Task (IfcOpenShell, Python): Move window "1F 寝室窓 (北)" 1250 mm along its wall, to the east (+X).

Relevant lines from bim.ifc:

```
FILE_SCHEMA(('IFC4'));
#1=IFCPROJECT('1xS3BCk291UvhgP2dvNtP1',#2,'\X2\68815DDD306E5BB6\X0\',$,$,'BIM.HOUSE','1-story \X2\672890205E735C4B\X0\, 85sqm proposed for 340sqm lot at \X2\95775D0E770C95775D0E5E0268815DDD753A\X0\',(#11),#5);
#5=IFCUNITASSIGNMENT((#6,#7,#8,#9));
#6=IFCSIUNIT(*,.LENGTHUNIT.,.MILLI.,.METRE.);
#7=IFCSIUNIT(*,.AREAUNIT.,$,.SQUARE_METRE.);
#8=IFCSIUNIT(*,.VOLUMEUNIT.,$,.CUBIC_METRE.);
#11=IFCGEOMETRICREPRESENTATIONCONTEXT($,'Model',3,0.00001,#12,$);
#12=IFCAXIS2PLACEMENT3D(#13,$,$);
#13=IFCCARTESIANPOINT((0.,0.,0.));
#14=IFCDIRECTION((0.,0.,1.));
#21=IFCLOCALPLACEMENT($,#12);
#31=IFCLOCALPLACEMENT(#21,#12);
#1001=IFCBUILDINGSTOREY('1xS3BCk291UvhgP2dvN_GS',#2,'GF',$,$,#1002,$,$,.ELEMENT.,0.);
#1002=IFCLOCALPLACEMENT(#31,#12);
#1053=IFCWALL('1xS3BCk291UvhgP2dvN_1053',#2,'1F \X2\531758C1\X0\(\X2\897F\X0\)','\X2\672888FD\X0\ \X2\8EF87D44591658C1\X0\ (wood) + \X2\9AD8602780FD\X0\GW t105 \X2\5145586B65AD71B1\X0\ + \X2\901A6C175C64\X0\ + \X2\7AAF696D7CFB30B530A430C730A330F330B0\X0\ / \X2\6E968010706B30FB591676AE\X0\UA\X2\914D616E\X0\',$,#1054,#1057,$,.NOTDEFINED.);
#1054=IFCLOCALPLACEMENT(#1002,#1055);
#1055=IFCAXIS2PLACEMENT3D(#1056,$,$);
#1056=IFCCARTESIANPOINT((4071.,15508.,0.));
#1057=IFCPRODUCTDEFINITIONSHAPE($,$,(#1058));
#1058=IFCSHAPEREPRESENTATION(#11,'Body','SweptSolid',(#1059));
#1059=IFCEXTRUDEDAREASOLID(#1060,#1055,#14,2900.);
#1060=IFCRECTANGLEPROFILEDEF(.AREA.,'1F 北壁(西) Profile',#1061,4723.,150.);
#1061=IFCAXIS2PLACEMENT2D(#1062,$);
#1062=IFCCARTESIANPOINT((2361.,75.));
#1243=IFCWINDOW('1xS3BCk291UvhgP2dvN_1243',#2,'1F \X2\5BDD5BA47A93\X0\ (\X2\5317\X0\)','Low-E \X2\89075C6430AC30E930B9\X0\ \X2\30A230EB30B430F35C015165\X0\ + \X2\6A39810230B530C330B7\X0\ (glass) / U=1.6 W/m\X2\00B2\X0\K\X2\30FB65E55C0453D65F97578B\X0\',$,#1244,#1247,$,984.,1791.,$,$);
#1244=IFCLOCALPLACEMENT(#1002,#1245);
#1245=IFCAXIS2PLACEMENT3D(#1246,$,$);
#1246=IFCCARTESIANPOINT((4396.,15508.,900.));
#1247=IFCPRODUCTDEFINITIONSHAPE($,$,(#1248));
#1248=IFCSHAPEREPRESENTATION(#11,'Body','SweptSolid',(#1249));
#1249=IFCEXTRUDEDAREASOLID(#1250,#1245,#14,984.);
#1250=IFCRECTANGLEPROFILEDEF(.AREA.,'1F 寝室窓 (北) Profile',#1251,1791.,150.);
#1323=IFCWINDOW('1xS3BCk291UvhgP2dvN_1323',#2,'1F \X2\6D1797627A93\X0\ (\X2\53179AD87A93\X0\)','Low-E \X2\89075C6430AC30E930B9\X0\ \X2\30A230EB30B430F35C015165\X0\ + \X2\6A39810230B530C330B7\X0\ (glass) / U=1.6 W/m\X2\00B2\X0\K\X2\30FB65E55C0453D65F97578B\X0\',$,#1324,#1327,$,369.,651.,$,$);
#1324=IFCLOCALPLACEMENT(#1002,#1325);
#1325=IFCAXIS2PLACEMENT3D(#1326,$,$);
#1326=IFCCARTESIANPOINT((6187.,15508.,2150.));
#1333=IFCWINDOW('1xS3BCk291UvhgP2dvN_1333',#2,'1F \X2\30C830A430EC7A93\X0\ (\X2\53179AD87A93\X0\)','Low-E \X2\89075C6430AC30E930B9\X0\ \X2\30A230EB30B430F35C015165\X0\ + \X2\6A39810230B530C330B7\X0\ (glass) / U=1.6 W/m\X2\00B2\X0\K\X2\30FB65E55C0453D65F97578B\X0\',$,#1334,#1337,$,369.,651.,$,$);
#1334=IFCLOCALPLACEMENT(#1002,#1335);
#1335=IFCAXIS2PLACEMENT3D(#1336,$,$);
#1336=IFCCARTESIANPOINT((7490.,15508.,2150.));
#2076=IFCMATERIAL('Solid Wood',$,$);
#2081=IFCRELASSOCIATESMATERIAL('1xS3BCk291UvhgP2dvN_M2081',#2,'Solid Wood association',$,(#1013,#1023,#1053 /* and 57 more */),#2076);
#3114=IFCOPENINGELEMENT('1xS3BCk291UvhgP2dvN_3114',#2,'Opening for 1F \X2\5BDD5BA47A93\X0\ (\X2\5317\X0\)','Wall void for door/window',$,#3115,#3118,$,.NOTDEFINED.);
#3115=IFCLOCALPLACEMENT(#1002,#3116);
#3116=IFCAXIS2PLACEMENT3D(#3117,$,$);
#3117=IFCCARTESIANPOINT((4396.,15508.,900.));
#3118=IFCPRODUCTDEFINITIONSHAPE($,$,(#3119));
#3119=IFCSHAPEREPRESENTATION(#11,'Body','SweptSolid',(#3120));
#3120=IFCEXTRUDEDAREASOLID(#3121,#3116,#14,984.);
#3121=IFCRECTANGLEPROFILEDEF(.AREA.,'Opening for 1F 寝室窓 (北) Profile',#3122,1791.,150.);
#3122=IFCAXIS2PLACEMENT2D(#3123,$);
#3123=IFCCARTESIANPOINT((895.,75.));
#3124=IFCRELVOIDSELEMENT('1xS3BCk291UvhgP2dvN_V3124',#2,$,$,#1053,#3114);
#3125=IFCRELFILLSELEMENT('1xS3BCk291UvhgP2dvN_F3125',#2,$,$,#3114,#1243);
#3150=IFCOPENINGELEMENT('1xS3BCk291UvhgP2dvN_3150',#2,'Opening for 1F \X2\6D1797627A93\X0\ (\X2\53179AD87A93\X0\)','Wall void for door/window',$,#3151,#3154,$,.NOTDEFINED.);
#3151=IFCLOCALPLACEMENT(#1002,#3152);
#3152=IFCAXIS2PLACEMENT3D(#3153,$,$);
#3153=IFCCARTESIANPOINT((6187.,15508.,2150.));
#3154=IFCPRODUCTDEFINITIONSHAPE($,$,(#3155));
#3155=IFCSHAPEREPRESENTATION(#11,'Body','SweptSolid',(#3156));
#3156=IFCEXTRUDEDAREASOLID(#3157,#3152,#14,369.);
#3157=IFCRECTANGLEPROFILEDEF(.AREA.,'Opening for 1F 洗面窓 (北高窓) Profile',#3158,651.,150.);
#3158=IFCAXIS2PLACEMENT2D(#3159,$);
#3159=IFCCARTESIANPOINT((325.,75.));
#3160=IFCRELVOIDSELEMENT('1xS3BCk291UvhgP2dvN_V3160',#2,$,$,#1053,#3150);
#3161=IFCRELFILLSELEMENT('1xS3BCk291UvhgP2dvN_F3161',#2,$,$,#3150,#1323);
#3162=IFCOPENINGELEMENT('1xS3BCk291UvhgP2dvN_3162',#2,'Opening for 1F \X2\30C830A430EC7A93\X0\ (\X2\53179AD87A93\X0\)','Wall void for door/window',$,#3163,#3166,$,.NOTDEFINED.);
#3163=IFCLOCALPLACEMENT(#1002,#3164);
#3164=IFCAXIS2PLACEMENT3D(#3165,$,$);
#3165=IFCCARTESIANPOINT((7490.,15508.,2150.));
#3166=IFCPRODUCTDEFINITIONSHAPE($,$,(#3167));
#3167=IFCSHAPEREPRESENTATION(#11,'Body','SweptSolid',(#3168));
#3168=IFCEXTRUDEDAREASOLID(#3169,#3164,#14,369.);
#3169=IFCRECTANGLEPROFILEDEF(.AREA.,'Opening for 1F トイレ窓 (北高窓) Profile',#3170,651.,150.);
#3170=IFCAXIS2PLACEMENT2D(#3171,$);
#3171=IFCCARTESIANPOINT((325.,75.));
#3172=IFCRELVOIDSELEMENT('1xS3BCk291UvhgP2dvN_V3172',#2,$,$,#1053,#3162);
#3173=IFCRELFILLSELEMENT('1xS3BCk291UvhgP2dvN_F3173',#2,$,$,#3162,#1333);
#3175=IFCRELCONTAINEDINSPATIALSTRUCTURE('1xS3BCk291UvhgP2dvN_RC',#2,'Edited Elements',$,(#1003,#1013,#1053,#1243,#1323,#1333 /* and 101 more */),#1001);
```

```python
import ifcopenshell
import ifcopenshell.api.geometry
import ifcopenshell.util.placement
import ifcopenshell.util.unit

model = ifcopenshell.open("bim.ifc")
unit_scale = ifcopenshell.util.unit.calculate_unit_scale(model)

window = model.by_id(1243)
opening = window.FillsVoids[0].RelatingOpeningElement
wall = opening.VoidsElements[0].RelatingBuildingElement

wall_matrix = ifcopenshell.util.placement.get_local_placement(wall.ObjectPlacement)
shift = wall_matrix[:3, 0] * 1.25 / unit_scale
before = ifcopenshell.util.placement.get_local_placement(window.ObjectPlacement)[:3, 3].copy()

# The window is not placed relative to its opening, so move both.
for product in (opening, window):
    matrix = ifcopenshell.util.placement.get_local_placement(product.ObjectPlacement)
    matrix[:3, 3] += shift
    ifcopenshell.api.geometry.edit_object_placement(model, product=product, matrix=matrix, is_si=False)

after = ifcopenshell.util.placement.get_local_placement(window.ObjectPlacement)[:3, 3]
print("window moved by", (after - before).round(3) + 0.0)

model.write("bim_v2.ifc")
```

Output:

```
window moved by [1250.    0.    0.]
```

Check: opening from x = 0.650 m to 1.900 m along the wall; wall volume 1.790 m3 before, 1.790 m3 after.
